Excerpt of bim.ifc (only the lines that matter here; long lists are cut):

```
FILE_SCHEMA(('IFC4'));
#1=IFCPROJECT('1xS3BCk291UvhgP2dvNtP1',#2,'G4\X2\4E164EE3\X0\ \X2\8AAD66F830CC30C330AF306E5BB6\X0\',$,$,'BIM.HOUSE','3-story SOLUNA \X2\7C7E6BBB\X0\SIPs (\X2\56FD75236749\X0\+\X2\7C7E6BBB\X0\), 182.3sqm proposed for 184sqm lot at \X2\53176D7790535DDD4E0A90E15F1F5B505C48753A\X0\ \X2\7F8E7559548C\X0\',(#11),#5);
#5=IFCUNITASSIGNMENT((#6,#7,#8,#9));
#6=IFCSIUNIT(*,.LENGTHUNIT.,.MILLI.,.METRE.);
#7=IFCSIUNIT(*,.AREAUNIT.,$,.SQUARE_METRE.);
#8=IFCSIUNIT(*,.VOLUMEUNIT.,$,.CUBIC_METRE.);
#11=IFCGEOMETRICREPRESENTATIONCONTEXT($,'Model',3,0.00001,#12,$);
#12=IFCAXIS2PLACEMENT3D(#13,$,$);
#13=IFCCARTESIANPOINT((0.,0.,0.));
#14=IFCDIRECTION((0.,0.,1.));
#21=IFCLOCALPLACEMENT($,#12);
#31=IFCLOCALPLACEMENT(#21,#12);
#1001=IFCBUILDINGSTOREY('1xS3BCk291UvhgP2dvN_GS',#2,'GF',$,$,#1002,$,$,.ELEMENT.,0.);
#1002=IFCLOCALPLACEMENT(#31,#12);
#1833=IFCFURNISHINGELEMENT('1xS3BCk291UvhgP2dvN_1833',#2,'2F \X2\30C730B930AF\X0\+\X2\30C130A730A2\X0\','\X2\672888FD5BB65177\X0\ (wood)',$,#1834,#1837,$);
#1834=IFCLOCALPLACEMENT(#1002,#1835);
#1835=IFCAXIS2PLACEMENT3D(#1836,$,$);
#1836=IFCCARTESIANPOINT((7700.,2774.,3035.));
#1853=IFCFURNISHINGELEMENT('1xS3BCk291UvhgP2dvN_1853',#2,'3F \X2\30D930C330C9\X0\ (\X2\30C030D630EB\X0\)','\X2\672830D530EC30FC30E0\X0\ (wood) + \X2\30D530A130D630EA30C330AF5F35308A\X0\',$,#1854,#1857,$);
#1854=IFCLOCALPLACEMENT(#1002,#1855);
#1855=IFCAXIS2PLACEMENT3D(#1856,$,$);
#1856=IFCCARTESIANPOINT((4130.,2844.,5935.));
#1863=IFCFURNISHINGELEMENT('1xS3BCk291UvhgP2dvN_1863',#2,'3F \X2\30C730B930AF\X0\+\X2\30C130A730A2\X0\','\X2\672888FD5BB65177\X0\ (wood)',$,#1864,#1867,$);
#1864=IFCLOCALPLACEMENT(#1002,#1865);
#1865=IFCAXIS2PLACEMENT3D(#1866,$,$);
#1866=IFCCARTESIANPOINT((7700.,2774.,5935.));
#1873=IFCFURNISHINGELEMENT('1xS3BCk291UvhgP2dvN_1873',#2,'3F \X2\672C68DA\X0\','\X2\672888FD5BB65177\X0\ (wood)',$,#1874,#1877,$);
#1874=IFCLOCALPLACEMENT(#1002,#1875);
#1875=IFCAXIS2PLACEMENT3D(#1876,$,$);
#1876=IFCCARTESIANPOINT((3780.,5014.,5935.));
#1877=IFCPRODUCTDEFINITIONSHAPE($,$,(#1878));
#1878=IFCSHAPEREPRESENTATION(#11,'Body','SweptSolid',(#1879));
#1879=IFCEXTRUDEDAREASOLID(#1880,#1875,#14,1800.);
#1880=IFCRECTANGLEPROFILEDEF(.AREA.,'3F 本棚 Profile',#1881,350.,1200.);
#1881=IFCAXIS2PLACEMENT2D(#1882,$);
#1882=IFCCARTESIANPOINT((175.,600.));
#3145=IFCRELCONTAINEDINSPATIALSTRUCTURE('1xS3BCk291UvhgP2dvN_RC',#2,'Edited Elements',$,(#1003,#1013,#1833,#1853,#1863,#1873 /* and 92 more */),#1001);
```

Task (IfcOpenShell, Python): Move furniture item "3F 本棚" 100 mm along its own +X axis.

```python
import ifcopenshell
import ifcopenshell.api.geometry
import ifcopenshell.util.placement
import ifcopenshell.util.unit

model = ifcopenshell.open("bim.ifc")
unit_scale = ifcopenshell.util.unit.calculate_unit_scale(model)

item = model.by_id(1873)
matrix = ifcopenshell.util.placement.get_local_placement(item.ObjectPlacement)
matrix[:3, 3] += matrix[:3, 0] * 0.1 / unit_scale
ifcopenshell.api.geometry.edit_object_placement(model, product=item, matrix=matrix, is_si=False)

print(ifcopenshell.util.placement.get_local_placement(item.ObjectPlacement).round(3) + 0.0)

model.write("bim-out.ifc")
```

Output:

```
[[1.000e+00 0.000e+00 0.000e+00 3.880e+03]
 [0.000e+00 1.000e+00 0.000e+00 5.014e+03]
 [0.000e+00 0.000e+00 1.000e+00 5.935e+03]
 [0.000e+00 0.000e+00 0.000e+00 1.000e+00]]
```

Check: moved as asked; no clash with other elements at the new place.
